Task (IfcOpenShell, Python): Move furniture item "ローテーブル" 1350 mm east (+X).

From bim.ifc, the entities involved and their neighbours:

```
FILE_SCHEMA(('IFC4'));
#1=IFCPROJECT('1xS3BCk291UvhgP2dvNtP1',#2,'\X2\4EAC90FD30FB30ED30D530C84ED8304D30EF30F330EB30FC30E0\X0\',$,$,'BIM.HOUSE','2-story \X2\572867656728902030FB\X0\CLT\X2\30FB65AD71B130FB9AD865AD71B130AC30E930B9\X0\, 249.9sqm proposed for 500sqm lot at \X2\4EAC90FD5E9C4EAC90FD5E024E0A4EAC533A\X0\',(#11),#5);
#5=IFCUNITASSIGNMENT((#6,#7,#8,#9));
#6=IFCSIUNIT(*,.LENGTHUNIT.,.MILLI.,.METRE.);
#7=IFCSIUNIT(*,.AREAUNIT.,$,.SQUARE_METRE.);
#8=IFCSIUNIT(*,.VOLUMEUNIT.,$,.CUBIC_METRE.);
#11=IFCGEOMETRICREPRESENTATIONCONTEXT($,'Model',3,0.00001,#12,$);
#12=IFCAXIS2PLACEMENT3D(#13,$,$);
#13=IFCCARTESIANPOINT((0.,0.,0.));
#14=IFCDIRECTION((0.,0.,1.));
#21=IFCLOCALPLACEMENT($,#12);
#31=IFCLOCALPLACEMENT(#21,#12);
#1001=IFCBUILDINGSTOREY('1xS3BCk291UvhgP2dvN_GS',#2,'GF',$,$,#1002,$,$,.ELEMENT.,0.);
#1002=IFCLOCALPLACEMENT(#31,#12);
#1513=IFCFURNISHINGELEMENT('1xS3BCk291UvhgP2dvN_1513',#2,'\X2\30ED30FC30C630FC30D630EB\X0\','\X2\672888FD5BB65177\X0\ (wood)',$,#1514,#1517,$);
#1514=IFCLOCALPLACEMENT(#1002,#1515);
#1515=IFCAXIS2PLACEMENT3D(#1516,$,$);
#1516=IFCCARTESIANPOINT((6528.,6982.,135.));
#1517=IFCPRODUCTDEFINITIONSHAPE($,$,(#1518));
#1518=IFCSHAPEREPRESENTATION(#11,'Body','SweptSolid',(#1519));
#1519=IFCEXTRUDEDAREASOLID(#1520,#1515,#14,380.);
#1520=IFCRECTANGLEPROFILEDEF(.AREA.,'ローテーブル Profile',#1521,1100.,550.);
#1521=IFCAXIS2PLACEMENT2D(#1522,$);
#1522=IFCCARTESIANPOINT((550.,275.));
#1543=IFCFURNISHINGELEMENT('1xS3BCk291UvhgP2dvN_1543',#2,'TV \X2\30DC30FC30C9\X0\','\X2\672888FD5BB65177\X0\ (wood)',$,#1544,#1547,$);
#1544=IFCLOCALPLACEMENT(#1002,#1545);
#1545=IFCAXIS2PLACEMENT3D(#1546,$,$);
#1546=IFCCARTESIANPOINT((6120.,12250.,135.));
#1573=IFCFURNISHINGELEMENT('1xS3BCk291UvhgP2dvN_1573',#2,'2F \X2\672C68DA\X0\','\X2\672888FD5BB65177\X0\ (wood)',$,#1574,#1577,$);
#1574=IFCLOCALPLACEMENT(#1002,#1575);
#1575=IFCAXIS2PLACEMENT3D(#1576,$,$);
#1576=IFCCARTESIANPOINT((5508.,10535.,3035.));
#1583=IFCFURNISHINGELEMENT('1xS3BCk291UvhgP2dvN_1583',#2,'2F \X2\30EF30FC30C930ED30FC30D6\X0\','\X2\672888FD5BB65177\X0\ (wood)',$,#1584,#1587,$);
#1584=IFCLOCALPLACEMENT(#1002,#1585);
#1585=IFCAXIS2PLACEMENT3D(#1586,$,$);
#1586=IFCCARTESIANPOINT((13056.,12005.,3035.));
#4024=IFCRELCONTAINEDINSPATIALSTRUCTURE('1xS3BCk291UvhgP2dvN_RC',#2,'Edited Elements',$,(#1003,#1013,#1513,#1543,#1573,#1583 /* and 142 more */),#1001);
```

```python
import ifcopenshell
import ifcopenshell.api.geometry
import ifcopenshell.util.placement
import ifcopenshell.util.unit

model = ifcopenshell.open("bim.ifc")
unit_scale = ifcopenshell.util.unit.calculate_unit_scale(model)

item = model.by_guid("1xS3BCk291UvhgP2dvN_1513")
matrix = ifcopenshell.util.placement.get_local_placement(item.ObjectPlacement)
matrix[0, 3] += 1.35 / unit_scale
ifcopenshell.api.geometry.edit_object_placement(model, product=item, matrix=matrix, is_si=False)

print(ifcopenshell.util.placement.get_local_placement(item.ObjectPlacement).round(3) + 0.0)

model.write("bim-out.ifc")
```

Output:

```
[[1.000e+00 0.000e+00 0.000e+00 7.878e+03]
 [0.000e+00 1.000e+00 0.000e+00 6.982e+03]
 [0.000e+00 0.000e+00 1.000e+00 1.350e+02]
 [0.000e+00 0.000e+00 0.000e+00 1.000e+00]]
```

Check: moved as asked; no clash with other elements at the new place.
